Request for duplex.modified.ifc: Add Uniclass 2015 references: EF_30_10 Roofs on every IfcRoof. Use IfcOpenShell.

First a look at what the model holds.

```python
import ifcopenshell

model = ifcopenshell.open("duplex.modified.ifc")
print(model.schema)
print("classifications:", [c.Name for c in model.by_type("IfcClassification")])
for ifc_class in ("IfcDoor", "IfcRoof", "IfcStair", "IfcWall", "IfcWindow"):
    print(ifc_class, len(model.by_type(ifc_class)))
```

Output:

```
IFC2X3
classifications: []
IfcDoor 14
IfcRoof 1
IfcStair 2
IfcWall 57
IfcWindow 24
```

```python
import ifcopenshell
import ifcopenshell.api.classification

model = ifcopenshell.open("duplex.modified.ifc")

# IFC2X3 requires Source and Edition and has no link from the project to the system.
system = model.create_entity("IfcClassification", Source="NBS", Edition="2015", Name="Uniclass 2015")

codes = {
    "IfcRoof": ("EF_30_10", "Roofs"),
}
for ifc_class, (code, name) in codes.items():
    products = model.by_type(ifc_class)
    ifcopenshell.api.classification.add_reference(
        model, products=products, classification=system, identification=code, name=name
    )
    print(code, len(products))

model.write("duplex.modified-out.ifc")
```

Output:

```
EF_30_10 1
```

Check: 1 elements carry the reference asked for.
